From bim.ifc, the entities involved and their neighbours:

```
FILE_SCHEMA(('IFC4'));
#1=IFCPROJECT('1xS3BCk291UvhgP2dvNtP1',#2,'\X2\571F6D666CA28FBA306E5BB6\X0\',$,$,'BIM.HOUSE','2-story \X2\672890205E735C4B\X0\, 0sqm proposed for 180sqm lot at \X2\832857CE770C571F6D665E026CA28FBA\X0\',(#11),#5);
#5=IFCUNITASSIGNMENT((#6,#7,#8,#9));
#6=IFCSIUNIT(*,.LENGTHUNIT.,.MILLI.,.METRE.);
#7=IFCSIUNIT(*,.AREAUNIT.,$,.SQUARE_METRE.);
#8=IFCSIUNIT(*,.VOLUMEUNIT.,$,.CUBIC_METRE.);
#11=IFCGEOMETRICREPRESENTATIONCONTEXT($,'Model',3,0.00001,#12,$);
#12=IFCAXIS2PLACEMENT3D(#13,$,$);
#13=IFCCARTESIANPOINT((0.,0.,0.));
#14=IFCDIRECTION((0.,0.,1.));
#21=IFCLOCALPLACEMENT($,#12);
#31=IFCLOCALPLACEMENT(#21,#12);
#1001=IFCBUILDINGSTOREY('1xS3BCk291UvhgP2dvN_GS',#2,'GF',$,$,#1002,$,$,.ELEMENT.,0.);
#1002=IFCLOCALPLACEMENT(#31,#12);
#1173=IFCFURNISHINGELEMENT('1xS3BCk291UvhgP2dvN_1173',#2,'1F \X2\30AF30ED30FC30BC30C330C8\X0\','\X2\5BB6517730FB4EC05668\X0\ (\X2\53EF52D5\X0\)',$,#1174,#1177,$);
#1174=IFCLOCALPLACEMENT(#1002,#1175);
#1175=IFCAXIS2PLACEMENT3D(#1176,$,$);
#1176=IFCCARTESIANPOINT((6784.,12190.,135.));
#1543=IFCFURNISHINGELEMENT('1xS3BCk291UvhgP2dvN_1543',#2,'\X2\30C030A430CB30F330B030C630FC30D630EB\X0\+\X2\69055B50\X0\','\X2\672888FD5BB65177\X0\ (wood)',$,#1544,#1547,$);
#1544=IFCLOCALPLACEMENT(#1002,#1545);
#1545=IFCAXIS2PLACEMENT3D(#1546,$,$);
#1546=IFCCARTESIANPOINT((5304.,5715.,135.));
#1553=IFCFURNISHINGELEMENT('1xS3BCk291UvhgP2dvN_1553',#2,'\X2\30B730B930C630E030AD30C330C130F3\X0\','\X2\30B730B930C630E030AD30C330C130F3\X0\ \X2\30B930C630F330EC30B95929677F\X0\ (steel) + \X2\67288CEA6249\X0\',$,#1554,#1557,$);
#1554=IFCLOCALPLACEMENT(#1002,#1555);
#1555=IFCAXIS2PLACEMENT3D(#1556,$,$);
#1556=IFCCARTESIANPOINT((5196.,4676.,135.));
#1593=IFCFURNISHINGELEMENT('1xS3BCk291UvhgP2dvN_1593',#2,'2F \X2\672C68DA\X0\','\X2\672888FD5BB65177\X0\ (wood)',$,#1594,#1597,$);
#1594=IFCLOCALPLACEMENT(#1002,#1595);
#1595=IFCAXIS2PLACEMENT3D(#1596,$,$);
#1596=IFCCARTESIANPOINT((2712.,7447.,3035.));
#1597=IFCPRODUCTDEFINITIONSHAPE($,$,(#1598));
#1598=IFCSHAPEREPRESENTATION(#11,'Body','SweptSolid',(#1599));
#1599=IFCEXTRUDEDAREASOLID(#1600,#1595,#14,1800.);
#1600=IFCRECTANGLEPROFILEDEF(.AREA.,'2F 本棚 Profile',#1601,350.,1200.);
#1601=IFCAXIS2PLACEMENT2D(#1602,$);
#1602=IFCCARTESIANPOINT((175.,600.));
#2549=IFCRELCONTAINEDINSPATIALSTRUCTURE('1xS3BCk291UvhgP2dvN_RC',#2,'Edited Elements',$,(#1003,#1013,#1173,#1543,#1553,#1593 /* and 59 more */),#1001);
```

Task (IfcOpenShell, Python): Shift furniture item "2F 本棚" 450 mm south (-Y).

```python
import ifcopenshell
import ifcopenshell.api.geometry
import ifcopenshell.util.placement

model = ifcopenshell.open("bim.ifc")

item = model.by_guid("1xS3BCk291UvhgP2dvN_1593")
matrix = ifcopenshell.util.placement.get_local_placement(item.ObjectPlacement)
matrix[1, 3] -= 450.0
ifcopenshell.api.geometry.edit_object_placement(model, product=item, matrix=matrix, is_si=False)

print(ifcopenshell.util.placement.get_local_placement(item.ObjectPlacement).round(3) + 0.0)

model.write("bim-out.ifc")
```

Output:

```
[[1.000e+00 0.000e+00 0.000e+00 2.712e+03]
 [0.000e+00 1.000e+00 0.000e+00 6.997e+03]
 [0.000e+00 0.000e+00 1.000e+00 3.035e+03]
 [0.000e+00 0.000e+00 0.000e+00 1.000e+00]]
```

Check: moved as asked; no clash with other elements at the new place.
